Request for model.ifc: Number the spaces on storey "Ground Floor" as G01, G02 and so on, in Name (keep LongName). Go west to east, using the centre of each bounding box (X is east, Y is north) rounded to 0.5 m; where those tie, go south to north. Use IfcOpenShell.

First a look at what the model holds.

```python
import ifcopenshell
import ifcopenshell.util.element
import ifcopenshell.util.placement

model = ifcopenshell.open("model.ifc")
print(model.schema)
storey = next(s for s in model.by_type("IfcBuildingStorey") if s.Name == "Ground Floor")
spaces = [e for e in ifcopenshell.util.element.get_decomposition(storey) if e.is_a("IfcSpace")]
for e in sorted(spaces, key=lambda e: e.id()):
    origin = ifcopenshell.util.placement.get_local_placement(e.ObjectPlacement)[:3, 3]
    print(e.id(), e.Name, e.LongName, origin.round(2) + 0.0, sep=" | ")
```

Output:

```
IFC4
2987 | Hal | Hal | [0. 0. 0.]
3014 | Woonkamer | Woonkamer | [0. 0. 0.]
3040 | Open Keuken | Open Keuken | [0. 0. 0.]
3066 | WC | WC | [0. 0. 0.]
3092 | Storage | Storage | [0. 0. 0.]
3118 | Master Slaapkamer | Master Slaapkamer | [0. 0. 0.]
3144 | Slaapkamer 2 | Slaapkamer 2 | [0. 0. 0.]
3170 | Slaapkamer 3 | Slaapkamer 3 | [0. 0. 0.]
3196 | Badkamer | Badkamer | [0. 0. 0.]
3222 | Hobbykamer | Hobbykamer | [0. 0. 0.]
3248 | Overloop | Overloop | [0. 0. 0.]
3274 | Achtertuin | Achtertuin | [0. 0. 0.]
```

```python
import ifcopenshell
import ifcopenshell.geom
import ifcopenshell.util.element
import ifcopenshell.util.shape

model = ifcopenshell.open("model.ifc")
settings = ifcopenshell.geom.settings()
settings.set("use-world-coords", True)


def centre(element):
    shape = ifcopenshell.geom.create_shape(settings, element)
    return ifcopenshell.util.shape.get_bbox_centroid(shape.geometry)


storey = next(s for s in model.by_type("IfcBuildingStorey") if s.Name == "Ground Floor")
spaces = [e for e in ifcopenshell.util.element.get_decomposition(storey) if e.is_a("IfcSpace")]

# Insertion points can sit at a corner or the storey origin, so sort by the geometry (in metres).
centres = {e: centre(e) for e in spaces}
spaces.sort(key=lambda e: (round(centres[e][0] / 0.5), centres[e][1]))

for i, e in enumerate(spaces, start=1):
    number = f"G{i:02d}"
    e.Name = number
    print(e.id(), number)

model.write("model_rev.ifc")
```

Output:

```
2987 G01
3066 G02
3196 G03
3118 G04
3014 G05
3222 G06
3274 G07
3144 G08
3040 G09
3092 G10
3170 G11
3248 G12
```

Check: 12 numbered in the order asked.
